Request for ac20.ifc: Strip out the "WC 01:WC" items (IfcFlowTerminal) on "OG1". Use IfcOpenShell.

First a look at what the model holds.

```python
import ifcopenshell
import ifcopenshell.util.element

model = ifcopenshell.open("ac20.ifc")
print(model.schema)
storey = next(s for s in model.by_type("IfcBuildingStorey") if s.Name == "OG1")
terminals = [e for e in ifcopenshell.util.element.get_decomposition(storey) if e.is_a("IfcFlowTerminal")]
seen = {}
for e in terminals:
    element_type = ifcopenshell.util.element.get_type(e)
    name = element_type.Name if element_type not in (None, e) else None
    seen[name] = seen.get(name, 0) + 1
for name, count in sorted(seen.items(), key=str):
    print(count, "x", name)
```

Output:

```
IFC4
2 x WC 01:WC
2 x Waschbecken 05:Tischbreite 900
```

```python
import ifcopenshell
import ifcopenshell.api.root
import ifcopenshell.util.element

model = ifcopenshell.open("ac20.ifc")

storey = next(s for s in model.by_type("IfcBuildingStorey") if s.Name == "OG1")
terminals = [e for e in ifcopenshell.util.element.get_decomposition(storey) if e.is_a("IfcFlowTerminal")]
targets = [e for e in terminals if (t := ifcopenshell.util.element.get_type(e)) not in (None, e) and t.Name == "WC 01:WC"]

for e in targets:
    ifcopenshell.api.root.remove_product(model, product=e)
print(len(targets), "removed")

model.write("ac20_updated.ifc")
```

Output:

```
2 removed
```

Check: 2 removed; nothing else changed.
